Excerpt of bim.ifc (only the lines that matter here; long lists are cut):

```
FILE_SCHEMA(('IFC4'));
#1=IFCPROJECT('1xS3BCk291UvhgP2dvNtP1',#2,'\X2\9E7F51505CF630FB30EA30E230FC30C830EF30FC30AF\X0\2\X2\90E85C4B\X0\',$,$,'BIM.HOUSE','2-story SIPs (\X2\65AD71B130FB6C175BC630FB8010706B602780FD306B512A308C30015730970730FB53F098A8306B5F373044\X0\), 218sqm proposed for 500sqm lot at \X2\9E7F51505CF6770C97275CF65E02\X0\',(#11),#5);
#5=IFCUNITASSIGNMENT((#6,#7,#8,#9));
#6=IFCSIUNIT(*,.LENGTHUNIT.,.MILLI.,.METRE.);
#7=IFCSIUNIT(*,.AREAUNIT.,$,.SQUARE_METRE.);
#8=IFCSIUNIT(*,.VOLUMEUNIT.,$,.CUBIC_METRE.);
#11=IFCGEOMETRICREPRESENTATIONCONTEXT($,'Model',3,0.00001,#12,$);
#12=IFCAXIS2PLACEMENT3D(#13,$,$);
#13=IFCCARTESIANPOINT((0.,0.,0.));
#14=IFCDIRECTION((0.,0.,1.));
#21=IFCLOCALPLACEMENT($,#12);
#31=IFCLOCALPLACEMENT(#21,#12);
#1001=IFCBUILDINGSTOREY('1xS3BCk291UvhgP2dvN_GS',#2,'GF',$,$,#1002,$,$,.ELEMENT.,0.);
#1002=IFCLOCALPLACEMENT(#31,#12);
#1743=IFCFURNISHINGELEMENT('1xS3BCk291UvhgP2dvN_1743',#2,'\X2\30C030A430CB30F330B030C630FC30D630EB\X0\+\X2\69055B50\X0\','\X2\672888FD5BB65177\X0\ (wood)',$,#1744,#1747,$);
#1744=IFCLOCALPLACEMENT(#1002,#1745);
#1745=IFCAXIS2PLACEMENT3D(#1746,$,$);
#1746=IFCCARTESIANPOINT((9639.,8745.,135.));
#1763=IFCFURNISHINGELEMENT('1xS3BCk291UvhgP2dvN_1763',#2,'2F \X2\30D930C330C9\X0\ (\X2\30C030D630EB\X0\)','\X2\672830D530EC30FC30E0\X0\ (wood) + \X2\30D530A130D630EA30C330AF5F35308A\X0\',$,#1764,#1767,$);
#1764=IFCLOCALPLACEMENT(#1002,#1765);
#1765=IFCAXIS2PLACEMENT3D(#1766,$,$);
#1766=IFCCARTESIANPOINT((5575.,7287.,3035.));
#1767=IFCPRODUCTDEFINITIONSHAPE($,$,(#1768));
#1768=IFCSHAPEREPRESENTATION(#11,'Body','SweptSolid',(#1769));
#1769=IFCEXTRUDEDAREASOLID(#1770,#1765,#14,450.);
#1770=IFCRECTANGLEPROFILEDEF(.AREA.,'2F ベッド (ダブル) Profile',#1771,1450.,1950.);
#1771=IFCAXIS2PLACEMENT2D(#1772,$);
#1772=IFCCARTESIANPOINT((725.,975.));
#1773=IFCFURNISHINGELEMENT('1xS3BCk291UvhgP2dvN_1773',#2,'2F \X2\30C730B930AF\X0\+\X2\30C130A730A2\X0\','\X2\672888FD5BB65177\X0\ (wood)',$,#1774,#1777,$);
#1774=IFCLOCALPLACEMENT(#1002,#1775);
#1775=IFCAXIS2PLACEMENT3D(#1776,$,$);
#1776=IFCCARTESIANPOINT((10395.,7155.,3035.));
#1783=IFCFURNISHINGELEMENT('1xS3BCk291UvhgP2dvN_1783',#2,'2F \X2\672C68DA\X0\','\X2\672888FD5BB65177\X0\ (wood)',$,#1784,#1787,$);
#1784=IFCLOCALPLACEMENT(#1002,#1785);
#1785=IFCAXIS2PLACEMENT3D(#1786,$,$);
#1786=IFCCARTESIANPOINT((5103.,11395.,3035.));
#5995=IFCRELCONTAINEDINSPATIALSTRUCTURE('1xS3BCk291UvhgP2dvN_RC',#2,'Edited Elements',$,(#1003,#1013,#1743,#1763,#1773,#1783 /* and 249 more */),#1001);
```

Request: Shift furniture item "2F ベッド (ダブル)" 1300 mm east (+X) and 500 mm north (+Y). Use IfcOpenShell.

```python
import ifcopenshell
import ifcopenshell.api.geometry
import ifcopenshell.util.placement

model = ifcopenshell.open("bim.ifc")

item = model.by_guid("1xS3BCk291UvhgP2dvN_1763")
matrix = ifcopenshell.util.placement.get_local_placement(item.ObjectPlacement)
matrix[0, 3] += 1300.0
matrix[1, 3] += 500.0
ifcopenshell.api.geometry.edit_object_placement(model, product=item, matrix=matrix, is_si=False)

print(ifcopenshell.util.placement.get_local_placement(item.ObjectPlacement).round(3) + 0.0)

model.write("bim_edited.ifc")
```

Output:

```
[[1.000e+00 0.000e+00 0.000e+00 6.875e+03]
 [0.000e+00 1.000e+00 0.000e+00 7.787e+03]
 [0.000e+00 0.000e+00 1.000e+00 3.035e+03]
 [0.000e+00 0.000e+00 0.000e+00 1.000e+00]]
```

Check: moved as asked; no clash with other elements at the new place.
